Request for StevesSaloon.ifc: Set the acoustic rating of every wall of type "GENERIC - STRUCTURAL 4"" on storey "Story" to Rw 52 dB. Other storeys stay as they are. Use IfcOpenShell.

First a look at what the model holds.

```python
import ifcopenshell
import ifcopenshell.util.element

model = ifcopenshell.open("StevesSaloon.ifc")
print(model.schema)
storey = next(s for s in model.by_type("IfcBuildingStorey") if s.Name == "Story")
walls = [e for e in ifcopenshell.util.element.get_decomposition(storey) if e.is_a("IfcWall")]
seen = {}
for e in walls:
    element_type = ifcopenshell.util.element.get_type(e)
    key = (element_type.Name if element_type != e and element_type else None, ifcopenshell.util.element.get_pset(e, "Pset_WallCommon", "AcousticRating"))
    seen[key] = seen.get(key, 0) + 1
for (name, value), count in sorted(seen.items(), key=str):
    print(count, "x", name, "|", value)
```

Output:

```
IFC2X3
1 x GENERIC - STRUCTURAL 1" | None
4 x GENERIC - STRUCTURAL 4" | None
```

```python
import ifcopenshell
import ifcopenshell.api.pset
import ifcopenshell.util.element

model = ifcopenshell.open("StevesSaloon.ifc")

storey = next(s for s in model.by_type("IfcBuildingStorey") if s.Name == "Story")
walls = [e for e in ifcopenshell.util.element.get_decomposition(storey) if e.is_a("IfcWall")]

count = 0
for e in walls:
    element_type = ifcopenshell.util.element.get_type(e)
    if element_type in (None, e) or element_type.Name != 'GENERIC - STRUCTURAL 4"':
        continue
    # add_pset returns the element's existing set when there is one.
    pset = ifcopenshell.api.pset.add_pset(model, product=e, name="Pset_WallCommon")
    ifcopenshell.api.pset.edit_pset(model, pset=pset, properties={"AcousticRating": "Rw 52 dB"})
    count += 1

print(count, "walls updated")

model.write("StevesSaloon_v2.ifc")
```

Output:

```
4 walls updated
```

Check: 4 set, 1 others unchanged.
